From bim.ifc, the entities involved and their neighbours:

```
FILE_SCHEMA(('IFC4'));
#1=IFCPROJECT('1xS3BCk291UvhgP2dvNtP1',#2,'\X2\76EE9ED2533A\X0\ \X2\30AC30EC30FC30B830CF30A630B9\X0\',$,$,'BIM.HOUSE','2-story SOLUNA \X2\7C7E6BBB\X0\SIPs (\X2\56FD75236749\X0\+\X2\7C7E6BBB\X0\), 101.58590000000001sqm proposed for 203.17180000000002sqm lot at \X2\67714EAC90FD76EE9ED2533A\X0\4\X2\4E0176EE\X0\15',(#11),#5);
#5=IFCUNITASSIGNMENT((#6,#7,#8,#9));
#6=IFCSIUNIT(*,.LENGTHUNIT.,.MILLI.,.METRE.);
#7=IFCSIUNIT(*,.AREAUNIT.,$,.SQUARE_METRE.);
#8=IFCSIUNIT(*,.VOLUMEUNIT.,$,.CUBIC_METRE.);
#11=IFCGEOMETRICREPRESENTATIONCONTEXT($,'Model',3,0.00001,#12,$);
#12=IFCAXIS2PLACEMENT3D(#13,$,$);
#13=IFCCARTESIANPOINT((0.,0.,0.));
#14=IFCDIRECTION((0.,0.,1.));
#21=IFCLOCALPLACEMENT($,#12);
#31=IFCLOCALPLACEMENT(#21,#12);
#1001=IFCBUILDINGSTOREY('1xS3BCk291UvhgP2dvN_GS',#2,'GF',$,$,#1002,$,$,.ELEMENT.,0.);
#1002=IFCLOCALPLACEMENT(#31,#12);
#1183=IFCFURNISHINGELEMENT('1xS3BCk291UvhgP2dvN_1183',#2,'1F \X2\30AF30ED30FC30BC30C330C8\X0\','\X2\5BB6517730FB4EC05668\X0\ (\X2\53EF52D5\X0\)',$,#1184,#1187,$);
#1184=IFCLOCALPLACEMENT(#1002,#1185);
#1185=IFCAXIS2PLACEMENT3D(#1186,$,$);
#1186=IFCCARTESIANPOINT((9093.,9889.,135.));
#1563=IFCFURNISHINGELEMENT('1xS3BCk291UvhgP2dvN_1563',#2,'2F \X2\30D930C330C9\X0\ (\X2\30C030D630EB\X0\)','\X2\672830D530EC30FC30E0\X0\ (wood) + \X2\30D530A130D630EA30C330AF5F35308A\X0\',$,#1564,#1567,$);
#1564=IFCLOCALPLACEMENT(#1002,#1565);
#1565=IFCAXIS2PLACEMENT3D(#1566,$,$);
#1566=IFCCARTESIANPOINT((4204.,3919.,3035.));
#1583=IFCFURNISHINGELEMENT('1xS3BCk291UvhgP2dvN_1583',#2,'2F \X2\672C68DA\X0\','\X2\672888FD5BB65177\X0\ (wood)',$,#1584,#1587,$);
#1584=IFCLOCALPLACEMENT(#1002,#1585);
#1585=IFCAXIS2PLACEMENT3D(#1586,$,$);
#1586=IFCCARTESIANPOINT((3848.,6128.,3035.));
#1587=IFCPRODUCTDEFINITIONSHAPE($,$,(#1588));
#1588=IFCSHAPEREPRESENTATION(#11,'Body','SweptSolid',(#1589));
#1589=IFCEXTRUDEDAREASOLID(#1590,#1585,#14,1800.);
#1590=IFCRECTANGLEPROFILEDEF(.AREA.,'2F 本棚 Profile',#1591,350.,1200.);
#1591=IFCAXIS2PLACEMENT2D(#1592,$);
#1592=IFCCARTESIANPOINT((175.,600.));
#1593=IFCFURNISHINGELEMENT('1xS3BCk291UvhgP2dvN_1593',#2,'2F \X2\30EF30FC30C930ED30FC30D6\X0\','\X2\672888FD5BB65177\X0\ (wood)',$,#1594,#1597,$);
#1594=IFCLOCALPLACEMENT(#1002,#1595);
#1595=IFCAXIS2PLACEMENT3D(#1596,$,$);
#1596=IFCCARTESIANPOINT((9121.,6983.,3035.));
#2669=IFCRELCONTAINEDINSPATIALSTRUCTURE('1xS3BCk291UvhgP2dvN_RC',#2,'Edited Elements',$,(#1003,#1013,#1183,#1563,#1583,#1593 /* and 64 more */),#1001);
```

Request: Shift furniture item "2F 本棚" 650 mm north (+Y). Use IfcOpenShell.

```python
import ifcopenshell
import ifcopenshell.api.geometry
import ifcopenshell.util.placement

model = ifcopenshell.open("bim.ifc")

item = model.by_id(1583)
matrix = ifcopenshell.util.placement.get_local_placement(item.ObjectPlacement)
matrix[1, 3] += 650.0
ifcopenshell.api.geometry.edit_object_placement(model, product=item, matrix=matrix, is_si=False)

print(ifcopenshell.util.placement.get_local_placement(item.ObjectPlacement).round(3) + 0.0)

model.write("bim_edited.ifc")
```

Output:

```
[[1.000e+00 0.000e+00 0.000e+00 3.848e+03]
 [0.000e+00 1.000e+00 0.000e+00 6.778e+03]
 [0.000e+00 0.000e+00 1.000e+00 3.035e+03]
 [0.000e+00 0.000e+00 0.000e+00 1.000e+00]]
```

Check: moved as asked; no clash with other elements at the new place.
